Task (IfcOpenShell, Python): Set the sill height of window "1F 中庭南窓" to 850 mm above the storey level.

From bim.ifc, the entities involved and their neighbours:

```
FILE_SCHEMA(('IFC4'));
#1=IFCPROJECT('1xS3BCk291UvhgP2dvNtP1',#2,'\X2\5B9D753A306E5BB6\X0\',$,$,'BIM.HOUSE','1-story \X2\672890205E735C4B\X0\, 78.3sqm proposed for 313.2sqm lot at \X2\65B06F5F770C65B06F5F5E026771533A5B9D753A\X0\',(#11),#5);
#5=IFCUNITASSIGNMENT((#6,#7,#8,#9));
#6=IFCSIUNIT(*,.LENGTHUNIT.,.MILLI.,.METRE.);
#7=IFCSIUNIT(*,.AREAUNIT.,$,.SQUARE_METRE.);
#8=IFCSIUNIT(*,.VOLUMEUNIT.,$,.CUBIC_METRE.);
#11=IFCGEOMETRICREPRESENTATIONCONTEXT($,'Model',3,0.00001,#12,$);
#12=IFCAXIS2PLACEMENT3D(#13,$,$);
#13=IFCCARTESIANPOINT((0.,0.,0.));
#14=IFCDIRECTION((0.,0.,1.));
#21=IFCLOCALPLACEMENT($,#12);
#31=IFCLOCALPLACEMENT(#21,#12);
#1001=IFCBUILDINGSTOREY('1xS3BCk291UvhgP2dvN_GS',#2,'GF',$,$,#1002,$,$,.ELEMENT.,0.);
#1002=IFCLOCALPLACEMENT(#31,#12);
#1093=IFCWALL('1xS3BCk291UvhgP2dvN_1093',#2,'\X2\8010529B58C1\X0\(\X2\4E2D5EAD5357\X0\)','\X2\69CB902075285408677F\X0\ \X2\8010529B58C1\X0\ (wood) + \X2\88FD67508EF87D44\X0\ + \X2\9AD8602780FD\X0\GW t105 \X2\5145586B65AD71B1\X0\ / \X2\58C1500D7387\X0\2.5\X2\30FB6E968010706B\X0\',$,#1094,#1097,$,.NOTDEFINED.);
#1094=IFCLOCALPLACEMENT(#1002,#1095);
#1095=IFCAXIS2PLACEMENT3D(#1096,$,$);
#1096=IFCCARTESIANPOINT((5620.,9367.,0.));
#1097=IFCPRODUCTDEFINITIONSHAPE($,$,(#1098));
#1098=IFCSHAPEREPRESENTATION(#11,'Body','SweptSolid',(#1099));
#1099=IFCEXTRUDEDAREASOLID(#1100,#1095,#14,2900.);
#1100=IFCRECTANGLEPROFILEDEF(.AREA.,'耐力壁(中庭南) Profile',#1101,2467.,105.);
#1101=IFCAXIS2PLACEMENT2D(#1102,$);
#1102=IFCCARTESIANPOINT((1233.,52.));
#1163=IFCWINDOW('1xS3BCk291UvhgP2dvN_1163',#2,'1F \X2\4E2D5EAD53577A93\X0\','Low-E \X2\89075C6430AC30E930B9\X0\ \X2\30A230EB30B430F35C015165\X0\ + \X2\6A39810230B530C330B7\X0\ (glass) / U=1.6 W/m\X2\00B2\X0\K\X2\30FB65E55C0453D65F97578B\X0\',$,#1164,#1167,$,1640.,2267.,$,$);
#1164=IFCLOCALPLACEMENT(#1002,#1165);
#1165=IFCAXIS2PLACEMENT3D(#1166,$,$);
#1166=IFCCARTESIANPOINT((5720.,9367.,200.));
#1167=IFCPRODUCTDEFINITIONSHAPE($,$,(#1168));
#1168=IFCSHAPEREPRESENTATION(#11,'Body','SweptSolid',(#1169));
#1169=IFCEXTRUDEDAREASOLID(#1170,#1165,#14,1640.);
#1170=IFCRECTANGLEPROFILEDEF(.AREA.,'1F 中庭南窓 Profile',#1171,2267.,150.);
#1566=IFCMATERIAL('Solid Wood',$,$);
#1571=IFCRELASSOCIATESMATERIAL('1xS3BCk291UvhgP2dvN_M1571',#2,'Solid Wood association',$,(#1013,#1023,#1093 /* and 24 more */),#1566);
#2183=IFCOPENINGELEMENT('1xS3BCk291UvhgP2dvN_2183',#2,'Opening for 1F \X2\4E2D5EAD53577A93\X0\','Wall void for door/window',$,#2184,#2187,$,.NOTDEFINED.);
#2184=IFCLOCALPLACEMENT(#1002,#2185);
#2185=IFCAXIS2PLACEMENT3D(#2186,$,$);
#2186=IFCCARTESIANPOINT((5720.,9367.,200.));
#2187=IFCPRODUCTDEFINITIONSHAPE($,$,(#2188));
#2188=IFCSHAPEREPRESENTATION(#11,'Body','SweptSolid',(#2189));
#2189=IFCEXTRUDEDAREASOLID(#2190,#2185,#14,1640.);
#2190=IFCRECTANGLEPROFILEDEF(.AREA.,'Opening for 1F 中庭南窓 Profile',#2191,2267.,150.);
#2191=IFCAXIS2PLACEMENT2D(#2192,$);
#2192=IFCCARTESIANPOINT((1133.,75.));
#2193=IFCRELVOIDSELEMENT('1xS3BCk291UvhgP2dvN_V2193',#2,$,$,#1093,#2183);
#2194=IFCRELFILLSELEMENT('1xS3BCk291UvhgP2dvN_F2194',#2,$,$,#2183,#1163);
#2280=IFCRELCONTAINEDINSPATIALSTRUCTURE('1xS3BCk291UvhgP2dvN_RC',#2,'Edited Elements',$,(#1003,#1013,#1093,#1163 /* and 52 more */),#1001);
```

```python
import numpy as np
import ifcopenshell
import ifcopenshell.api.geometry
import ifcopenshell.geom
import ifcopenshell.util.element
import ifcopenshell.util.placement
import ifcopenshell.util.shape
import ifcopenshell.util.unit

model = ifcopenshell.open("bim.ifc")
unit_scale = ifcopenshell.util.unit.calculate_unit_scale(model)

window = model.by_guid("1xS3BCk291UvhgP2dvN_1163")
opening = window.FillsVoids[0].RelatingOpeningElement
storey = ifcopenshell.util.element.get_container(window, ifc_class="IfcBuildingStorey")
level = ifcopenshell.util.placement.get_local_placement(storey.ObjectPlacement)[2, 3]

# The opening's origin need not be at the sill, so measure its lowest point.
shape = ifcopenshell.geom.create_shape(ifcopenshell.geom.settings(), opening)
bottom = ifcopenshell.util.shape.get_shape_bottom_elevation(shape, shape.geometry) / unit_scale
dz = level + 850.0 - bottom

shift = np.array([0.0, 0.0, dz])
# The window is not placed relative to its opening, so move both.
for product in (opening, window):
    matrix = ifcopenshell.util.placement.get_local_placement(product.ObjectPlacement)
    matrix[:3, 3] += shift
    ifcopenshell.api.geometry.edit_object_placement(model, product=product, matrix=matrix, is_si=False)

print(f"moved by {dz * unit_scale:+.3f} m")

model.write("bim_edited.ifc")
```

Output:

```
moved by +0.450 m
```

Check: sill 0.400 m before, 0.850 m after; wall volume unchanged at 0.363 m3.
